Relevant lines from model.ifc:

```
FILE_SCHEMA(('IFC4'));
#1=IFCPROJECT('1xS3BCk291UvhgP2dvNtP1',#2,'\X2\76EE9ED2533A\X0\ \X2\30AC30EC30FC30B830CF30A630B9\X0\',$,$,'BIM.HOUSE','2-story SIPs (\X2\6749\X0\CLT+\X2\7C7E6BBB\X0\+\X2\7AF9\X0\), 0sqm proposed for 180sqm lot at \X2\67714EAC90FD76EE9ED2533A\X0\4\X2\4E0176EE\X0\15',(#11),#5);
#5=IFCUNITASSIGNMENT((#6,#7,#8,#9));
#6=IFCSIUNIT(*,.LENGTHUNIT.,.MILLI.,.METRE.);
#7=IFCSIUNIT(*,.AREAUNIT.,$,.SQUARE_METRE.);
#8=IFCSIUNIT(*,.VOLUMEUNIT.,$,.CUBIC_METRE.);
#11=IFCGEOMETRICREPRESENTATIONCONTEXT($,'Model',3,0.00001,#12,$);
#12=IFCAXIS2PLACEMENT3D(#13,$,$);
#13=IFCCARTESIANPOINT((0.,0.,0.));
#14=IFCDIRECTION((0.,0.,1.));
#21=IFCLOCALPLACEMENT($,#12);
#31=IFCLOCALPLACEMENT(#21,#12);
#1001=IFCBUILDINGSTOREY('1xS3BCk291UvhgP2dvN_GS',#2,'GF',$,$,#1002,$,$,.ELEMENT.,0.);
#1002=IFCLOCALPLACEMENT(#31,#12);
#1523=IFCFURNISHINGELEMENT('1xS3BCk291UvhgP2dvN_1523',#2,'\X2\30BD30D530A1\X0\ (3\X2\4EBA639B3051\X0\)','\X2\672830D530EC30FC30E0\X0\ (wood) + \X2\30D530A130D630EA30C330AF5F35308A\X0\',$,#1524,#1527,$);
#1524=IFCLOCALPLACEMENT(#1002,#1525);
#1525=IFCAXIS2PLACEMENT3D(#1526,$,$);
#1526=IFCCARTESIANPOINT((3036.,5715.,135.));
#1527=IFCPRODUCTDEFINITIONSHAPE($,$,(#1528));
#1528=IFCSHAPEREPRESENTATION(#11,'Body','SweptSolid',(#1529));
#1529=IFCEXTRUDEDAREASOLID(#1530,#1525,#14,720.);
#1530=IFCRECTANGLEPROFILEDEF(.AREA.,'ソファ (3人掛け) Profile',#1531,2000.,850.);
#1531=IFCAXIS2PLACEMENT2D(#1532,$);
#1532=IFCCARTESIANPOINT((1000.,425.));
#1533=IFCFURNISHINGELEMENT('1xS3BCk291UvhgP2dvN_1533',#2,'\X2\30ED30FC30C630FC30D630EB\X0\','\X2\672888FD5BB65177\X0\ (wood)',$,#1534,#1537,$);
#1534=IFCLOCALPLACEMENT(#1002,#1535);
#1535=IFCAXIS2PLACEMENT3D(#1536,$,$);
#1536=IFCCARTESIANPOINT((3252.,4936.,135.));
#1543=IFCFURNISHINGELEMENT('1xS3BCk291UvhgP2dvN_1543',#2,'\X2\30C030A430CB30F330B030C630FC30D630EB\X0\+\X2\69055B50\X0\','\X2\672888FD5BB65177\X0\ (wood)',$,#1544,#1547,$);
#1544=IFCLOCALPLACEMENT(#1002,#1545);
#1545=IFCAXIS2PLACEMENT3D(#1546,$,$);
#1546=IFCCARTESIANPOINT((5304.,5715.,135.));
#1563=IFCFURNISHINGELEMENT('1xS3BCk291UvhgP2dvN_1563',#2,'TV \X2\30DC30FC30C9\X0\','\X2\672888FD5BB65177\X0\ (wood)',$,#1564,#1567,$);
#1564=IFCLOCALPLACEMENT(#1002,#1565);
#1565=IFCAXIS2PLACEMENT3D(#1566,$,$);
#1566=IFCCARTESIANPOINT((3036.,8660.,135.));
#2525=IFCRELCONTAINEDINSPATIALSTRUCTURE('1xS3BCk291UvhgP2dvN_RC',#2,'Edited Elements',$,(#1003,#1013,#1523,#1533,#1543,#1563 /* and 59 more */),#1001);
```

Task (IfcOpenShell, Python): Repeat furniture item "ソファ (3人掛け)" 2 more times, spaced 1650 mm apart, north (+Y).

```python
import numpy as np
import ifcopenshell
import ifcopenshell.api.geometry
import ifcopenshell.api.root
import ifcopenshell.util.element
import ifcopenshell.util.placement
import ifcopenshell.util.unit

model = ifcopenshell.open("model.ifc")
unit_scale = ifcopenshell.util.unit.calculate_unit_scale(model)


def reuse_history(source, copy):
    """copy_class also copies each property set's owner history, people and application; keep the originals."""
    for rel in copy.IsDefinedBy:
        if rel.is_a("IfcRelDefinesByProperties") and (history := rel.RelatingPropertyDefinition.OwnerHistory):
            rel.RelatingPropertyDefinition.OwnerHistory = source.OwnerHistory
            ifcopenshell.util.element.remove_deep2(model, history)


source = model.by_guid("1xS3BCk291UvhgP2dvN_1523")
base = ifcopenshell.util.placement.get_local_placement(source.ObjectPlacement)
step = np.array([0.0, 1.0, 0.0]) * 1.65 / unit_scale

for i in range(1, 3):
    copy = ifcopenshell.api.root.copy_class(model, product=source)
    copy.Representation = ifcopenshell.util.element.copy_deep(
        model, source.Representation, exclude=["IfcGeometricRepresentationContext", "IfcRepresentationMap"]
    )
    reuse_history(source, copy)
    matrix = base.copy()
    matrix[:3, 3] += i * step
    print("added at", matrix[:3, 3].round(3) + 0.0)
    ifcopenshell.api.geometry.edit_object_placement(model, product=copy, matrix=matrix, is_si=False)

model.write("model_edited.ifc")
```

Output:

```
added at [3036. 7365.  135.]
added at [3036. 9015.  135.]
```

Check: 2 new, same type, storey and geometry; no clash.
